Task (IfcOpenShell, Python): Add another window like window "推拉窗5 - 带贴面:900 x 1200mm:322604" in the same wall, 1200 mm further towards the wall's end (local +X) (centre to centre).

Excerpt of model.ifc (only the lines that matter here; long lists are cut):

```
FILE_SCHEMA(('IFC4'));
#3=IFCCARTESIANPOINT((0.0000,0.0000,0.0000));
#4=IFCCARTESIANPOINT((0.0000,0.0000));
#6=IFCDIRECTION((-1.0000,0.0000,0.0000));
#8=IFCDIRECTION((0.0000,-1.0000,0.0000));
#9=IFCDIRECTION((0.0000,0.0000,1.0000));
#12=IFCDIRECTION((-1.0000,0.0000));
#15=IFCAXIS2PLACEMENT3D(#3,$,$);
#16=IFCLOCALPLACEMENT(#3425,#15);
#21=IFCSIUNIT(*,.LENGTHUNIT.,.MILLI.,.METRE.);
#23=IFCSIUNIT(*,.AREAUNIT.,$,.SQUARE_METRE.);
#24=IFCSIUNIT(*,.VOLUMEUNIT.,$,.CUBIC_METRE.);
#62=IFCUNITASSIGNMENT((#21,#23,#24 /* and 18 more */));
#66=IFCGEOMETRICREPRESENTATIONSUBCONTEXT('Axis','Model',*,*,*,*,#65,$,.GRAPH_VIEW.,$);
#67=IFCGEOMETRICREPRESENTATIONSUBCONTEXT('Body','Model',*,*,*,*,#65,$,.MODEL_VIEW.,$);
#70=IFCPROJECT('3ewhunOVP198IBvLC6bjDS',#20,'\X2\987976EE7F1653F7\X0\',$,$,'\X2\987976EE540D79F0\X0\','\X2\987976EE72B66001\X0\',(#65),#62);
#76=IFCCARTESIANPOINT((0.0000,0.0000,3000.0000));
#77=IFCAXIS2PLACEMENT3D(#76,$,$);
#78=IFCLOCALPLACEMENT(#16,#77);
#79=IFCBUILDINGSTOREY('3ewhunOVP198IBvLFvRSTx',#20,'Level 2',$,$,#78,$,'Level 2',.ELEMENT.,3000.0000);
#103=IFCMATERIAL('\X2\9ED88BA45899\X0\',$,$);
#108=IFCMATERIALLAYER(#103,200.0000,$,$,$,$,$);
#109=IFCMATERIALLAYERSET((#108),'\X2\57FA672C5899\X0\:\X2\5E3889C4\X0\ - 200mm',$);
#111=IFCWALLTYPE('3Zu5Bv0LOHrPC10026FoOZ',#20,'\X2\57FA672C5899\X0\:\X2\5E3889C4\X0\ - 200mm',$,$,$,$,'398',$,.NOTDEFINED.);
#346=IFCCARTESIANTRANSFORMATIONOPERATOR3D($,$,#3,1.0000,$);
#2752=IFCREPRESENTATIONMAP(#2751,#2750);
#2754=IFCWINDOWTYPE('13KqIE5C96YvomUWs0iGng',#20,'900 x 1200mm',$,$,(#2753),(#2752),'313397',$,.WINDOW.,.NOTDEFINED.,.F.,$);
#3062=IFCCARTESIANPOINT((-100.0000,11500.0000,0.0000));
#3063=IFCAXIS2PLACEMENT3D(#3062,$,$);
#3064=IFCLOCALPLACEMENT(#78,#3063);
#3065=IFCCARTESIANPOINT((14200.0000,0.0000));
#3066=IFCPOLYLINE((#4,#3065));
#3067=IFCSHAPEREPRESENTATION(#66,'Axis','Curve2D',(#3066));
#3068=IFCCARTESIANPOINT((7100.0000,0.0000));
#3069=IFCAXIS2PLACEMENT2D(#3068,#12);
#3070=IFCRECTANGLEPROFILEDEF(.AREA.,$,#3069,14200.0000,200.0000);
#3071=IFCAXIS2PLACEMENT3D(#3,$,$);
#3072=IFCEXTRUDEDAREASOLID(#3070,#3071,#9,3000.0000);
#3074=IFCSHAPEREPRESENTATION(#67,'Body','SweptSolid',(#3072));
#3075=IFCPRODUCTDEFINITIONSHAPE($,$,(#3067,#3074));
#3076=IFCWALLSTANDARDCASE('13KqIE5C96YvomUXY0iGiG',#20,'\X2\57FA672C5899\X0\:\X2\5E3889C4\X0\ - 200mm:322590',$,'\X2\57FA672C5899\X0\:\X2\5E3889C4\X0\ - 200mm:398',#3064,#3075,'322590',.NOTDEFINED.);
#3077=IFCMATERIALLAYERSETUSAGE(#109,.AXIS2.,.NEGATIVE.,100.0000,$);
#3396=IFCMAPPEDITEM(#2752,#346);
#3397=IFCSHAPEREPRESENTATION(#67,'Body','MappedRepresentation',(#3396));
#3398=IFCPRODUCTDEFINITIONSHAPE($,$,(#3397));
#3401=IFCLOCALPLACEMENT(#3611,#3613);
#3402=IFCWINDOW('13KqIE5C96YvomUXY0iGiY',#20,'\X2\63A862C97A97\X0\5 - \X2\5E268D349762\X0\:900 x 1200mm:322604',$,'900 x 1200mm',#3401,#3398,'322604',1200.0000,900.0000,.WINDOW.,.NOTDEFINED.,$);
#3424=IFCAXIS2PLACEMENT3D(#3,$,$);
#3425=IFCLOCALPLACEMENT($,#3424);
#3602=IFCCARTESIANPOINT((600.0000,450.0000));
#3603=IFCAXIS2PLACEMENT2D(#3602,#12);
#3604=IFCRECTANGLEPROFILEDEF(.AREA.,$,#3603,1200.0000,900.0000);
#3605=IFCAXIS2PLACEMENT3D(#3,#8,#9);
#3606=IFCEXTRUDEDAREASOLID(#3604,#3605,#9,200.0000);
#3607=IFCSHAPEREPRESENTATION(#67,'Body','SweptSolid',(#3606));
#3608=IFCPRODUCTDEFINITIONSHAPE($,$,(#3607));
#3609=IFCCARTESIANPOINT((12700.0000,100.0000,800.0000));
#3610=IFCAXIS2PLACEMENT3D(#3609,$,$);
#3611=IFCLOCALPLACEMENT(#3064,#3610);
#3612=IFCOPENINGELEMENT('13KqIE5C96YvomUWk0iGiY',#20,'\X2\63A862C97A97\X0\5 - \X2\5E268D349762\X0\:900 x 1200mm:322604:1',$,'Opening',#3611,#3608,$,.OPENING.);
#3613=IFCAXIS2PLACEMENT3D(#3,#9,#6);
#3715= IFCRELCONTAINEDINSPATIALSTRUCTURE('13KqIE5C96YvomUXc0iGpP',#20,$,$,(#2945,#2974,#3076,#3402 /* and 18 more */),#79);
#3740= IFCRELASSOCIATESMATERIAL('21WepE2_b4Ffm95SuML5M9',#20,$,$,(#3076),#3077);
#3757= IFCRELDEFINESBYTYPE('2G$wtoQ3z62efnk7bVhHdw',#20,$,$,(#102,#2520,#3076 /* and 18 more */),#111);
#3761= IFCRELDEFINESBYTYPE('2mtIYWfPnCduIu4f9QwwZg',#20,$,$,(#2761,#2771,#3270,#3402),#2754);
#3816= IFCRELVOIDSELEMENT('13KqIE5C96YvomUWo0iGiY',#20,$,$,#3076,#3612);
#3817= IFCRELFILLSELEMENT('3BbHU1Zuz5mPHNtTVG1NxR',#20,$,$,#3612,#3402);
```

```python
import ifcopenshell
import ifcopenshell.api.feature
import ifcopenshell.api.geometry
import ifcopenshell.api.root
import ifcopenshell.geom
import ifcopenshell.util.element
import ifcopenshell.util.placement
import ifcopenshell.util.shape

model = ifcopenshell.open("model.ifc")
settings = ifcopenshell.geom.settings()


def volume(element):
    """Net volume in cubic metres, openings subtracted."""
    shape = ifcopenshell.geom.create_shape(settings, element)
    return ifcopenshell.util.shape.get_volume(shape.geometry)


def reuse_history(source, copy):
    """copy_class also copies each property set's owner history, people and application; keep the originals."""
    for rel in copy.IsDefinedBy:
        if rel.is_a("IfcRelDefinesByProperties") and (history := rel.RelatingPropertyDefinition.OwnerHistory):
            rel.RelatingPropertyDefinition.OwnerHistory = source.OwnerHistory
            ifcopenshell.util.element.remove_deep2(model, history)


window = model.by_guid("13KqIE5C96YvomUXY0iGiY")
opening = window.FillsVoids[0].RelatingOpeningElement
wall = opening.VoidsElements[0].RelatingBuildingElement
before = volume(wall)
shift = ifcopenshell.util.placement.get_local_placement(wall.ObjectPlacement)[:3, 0] * 1200.0

# copy_class copies the void relationship, type, container and properties, but no geometry.
new_opening = ifcopenshell.api.root.copy_class(model, product=opening)
new_opening.Representation = ifcopenshell.util.element.copy_deep(
    model, opening.Representation, exclude=["IfcGeometricRepresentationContext", "IfcRepresentationMap"]
)
new_opening.Name = "推拉窗5 - 带贴面:900 x 1200mm"
new_window = ifcopenshell.api.root.copy_class(model, product=window)
new_window.Representation = ifcopenshell.util.element.copy_deep(
    model, window.Representation, exclude=["IfcGeometricRepresentationContext", "IfcRepresentationMap"]
)
new_window.Name = "推拉窗5 - 带贴面:900 x 1200mm"
new_window.Tag = None
reuse_history(window, new_window)
ifcopenshell.api.feature.add_filling(model, opening=new_opening, element=new_window)

for old, new in ((opening, new_opening), (window, new_window)):
    matrix = ifcopenshell.util.placement.get_local_placement(old.ObjectPlacement)
    matrix[:3, 3] += shift
    ifcopenshell.api.geometry.edit_object_placement(model, product=new, matrix=matrix, is_si=False)

after = volume(wall)

print(f"wall volume {before:.3f} -> {after:.3f} m3")

model.write("model_updated.ifc")
```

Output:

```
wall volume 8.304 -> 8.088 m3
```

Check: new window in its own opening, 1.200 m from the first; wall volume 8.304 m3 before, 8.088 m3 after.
